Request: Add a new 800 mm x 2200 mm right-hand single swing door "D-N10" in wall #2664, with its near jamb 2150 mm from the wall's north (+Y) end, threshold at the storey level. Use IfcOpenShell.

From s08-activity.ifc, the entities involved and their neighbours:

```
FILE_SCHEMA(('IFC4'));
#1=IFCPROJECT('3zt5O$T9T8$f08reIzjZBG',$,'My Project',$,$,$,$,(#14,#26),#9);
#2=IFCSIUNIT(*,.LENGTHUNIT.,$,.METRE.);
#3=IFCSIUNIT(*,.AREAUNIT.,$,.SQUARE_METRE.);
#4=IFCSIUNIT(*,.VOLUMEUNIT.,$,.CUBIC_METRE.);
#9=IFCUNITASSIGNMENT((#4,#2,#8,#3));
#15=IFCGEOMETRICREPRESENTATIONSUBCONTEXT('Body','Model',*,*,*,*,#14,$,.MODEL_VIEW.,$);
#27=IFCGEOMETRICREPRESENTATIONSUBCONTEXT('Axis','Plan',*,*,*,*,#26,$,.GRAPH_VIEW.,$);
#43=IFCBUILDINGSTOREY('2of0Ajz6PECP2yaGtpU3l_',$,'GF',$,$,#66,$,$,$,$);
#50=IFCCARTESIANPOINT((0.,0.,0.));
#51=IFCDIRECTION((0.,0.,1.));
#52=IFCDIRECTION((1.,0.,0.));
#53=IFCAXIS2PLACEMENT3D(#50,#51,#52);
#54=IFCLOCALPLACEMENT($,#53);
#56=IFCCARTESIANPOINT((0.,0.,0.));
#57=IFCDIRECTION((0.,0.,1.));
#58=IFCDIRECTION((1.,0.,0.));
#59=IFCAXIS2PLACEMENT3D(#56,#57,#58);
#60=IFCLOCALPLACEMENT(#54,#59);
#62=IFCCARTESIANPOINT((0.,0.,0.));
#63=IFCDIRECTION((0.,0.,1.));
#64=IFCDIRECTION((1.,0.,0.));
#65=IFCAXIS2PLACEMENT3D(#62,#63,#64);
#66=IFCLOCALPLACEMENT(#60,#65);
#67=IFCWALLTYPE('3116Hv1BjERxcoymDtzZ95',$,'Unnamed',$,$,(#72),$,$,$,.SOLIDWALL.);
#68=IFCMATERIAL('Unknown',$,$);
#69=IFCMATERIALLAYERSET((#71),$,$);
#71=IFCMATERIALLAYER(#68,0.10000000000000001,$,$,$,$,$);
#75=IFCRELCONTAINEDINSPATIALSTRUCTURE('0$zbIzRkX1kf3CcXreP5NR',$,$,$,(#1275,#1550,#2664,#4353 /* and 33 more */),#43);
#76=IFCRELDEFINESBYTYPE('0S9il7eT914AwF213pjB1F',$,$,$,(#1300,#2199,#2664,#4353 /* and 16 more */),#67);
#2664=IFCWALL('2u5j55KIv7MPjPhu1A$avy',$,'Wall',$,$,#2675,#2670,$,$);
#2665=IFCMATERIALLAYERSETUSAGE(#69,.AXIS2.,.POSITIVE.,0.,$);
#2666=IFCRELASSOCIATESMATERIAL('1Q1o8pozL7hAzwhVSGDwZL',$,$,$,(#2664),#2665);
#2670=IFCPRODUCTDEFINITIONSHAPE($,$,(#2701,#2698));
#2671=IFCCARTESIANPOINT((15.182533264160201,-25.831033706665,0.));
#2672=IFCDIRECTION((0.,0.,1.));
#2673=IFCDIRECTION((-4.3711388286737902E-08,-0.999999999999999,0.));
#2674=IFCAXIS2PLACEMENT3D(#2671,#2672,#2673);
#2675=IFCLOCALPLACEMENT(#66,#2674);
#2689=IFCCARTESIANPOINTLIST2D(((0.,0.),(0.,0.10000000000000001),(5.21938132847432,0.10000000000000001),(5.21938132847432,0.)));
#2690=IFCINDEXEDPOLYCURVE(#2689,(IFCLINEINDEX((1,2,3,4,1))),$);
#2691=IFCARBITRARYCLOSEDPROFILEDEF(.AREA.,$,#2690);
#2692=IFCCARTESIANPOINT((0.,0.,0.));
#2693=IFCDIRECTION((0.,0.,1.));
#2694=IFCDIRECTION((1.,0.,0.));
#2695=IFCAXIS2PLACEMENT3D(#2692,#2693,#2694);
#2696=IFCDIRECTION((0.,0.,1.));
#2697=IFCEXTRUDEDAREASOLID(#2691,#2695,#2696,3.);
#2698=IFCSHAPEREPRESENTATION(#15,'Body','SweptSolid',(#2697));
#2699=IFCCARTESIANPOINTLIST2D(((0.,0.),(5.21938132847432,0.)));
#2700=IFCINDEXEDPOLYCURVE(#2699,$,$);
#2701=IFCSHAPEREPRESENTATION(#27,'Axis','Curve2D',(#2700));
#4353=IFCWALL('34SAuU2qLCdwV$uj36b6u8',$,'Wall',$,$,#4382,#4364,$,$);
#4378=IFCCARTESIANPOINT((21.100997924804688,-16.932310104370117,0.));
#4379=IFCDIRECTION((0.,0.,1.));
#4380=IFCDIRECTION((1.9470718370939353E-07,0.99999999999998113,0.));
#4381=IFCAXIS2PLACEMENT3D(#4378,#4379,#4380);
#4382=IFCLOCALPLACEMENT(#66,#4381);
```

```python
import numpy as np
import ifcopenshell
import ifcopenshell.api.feature
import ifcopenshell.api.geometry
import ifcopenshell.api.root
import ifcopenshell.api.spatial
import ifcopenshell.geom
import ifcopenshell.util.element
import ifcopenshell.util.placement
import ifcopenshell.util.representation
import ifcopenshell.util.shape
import ifcopenshell.util.unit

model = ifcopenshell.open("s08-activity.ifc")
unit_scale = ifcopenshell.util.unit.calculate_unit_scale(model)
settings = ifcopenshell.geom.settings()


def volume(element):
    """Net volume in cubic metres, openings subtracted."""
    shape = ifcopenshell.geom.create_shape(settings, element)
    return ifcopenshell.util.shape.get_volume(shape.geometry)


wall = model.by_guid("2u5j55KIv7MPjPhu1A$avy")
storey = ifcopenshell.util.element.get_container(wall, ifc_class="IfcBuildingStorey")
context = ifcopenshell.util.representation.get_context(model, "Model", "Body", "MODEL_VIEW")
before = volume(wall)

width, height, from_end, sill = 0.8, 2.2, 2.15, 0.0  # metres

# The wall runs along its own X axis, and the end named is its -X end.
wall_shape = ifcopenshell.geom.create_shape(settings, wall)
x, y, z = ifcopenshell.util.shape.get_vertices(wall_shape.geometry).T
start = x.min() + from_end
face, thickness = float(y.min()), float(y.max() - y.min())
wall_matrix = ifcopenshell.util.placement.get_local_placement(wall.ObjectPlacement)
level = ifcopenshell.util.placement.get_local_placement(storey.ObjectPlacement)[2, 3]


def in_wall(x, y):
    """Placement at x, y metres in the wall's axes, at sill height."""
    matrix = wall_matrix.copy()
    matrix[:, 3] = wall_matrix @ np.array([x / unit_scale, y / unit_scale, 0.0, 1.0])
    matrix[2, 3] = level + sill / unit_scale
    return matrix


# Opening: a box that overshoots both wall faces by 50 mm.
opening = ifcopenshell.api.root.create_entity(model, ifc_class="IfcOpeningElement", predefined_type="OPENING")
box = ifcopenshell.api.geometry.add_wall_representation(
    model, context=context, length=width, height=height, thickness=thickness + 0.1
)
ifcopenshell.api.geometry.assign_representation(model, product=opening, representation=box)
ifcopenshell.api.geometry.edit_object_placement(model, product=opening, matrix=in_wall(start, face - 0.05), is_si=False)
ifcopenshell.api.feature.add_feature(model, feature=opening, element=wall)

door = ifcopenshell.api.root.create_entity(model, ifc_class="IfcDoor", name="D-N10", predefined_type="DOOR")
door.OverallWidth, door.OverallHeight = width / unit_scale, height / unit_scale
door.OperationType = "SINGLE_SWING_RIGHT"
body = ifcopenshell.api.geometry.add_door_representation(
    model,
    context=context,
    overall_width=door.OverallWidth,
    overall_height=door.OverallHeight,
    operation_type="SINGLE_SWING_RIGHT",
    lining_properties={"LiningDepth": thickness / unit_scale, "ThresholdDepth": thickness / unit_scale},
)
ifcopenshell.api.geometry.assign_representation(model, product=door, representation=body)
ifcopenshell.api.spatial.assign_container(model, products=[door], relating_structure=storey)
ifcopenshell.api.feature.add_filling(model, opening=opening, element=door)

# The lining spans the wall, so the door starts at the wall face.
ifcopenshell.api.geometry.edit_object_placement(model, product=door, matrix=in_wall(start, face), is_si=False)

after = volume(wall)

print(f"wall volume {before:.3f} -> {after:.3f} m3")

model.write("s08-activity_updated.ifc")
```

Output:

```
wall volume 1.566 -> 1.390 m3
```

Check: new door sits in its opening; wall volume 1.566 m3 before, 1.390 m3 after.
